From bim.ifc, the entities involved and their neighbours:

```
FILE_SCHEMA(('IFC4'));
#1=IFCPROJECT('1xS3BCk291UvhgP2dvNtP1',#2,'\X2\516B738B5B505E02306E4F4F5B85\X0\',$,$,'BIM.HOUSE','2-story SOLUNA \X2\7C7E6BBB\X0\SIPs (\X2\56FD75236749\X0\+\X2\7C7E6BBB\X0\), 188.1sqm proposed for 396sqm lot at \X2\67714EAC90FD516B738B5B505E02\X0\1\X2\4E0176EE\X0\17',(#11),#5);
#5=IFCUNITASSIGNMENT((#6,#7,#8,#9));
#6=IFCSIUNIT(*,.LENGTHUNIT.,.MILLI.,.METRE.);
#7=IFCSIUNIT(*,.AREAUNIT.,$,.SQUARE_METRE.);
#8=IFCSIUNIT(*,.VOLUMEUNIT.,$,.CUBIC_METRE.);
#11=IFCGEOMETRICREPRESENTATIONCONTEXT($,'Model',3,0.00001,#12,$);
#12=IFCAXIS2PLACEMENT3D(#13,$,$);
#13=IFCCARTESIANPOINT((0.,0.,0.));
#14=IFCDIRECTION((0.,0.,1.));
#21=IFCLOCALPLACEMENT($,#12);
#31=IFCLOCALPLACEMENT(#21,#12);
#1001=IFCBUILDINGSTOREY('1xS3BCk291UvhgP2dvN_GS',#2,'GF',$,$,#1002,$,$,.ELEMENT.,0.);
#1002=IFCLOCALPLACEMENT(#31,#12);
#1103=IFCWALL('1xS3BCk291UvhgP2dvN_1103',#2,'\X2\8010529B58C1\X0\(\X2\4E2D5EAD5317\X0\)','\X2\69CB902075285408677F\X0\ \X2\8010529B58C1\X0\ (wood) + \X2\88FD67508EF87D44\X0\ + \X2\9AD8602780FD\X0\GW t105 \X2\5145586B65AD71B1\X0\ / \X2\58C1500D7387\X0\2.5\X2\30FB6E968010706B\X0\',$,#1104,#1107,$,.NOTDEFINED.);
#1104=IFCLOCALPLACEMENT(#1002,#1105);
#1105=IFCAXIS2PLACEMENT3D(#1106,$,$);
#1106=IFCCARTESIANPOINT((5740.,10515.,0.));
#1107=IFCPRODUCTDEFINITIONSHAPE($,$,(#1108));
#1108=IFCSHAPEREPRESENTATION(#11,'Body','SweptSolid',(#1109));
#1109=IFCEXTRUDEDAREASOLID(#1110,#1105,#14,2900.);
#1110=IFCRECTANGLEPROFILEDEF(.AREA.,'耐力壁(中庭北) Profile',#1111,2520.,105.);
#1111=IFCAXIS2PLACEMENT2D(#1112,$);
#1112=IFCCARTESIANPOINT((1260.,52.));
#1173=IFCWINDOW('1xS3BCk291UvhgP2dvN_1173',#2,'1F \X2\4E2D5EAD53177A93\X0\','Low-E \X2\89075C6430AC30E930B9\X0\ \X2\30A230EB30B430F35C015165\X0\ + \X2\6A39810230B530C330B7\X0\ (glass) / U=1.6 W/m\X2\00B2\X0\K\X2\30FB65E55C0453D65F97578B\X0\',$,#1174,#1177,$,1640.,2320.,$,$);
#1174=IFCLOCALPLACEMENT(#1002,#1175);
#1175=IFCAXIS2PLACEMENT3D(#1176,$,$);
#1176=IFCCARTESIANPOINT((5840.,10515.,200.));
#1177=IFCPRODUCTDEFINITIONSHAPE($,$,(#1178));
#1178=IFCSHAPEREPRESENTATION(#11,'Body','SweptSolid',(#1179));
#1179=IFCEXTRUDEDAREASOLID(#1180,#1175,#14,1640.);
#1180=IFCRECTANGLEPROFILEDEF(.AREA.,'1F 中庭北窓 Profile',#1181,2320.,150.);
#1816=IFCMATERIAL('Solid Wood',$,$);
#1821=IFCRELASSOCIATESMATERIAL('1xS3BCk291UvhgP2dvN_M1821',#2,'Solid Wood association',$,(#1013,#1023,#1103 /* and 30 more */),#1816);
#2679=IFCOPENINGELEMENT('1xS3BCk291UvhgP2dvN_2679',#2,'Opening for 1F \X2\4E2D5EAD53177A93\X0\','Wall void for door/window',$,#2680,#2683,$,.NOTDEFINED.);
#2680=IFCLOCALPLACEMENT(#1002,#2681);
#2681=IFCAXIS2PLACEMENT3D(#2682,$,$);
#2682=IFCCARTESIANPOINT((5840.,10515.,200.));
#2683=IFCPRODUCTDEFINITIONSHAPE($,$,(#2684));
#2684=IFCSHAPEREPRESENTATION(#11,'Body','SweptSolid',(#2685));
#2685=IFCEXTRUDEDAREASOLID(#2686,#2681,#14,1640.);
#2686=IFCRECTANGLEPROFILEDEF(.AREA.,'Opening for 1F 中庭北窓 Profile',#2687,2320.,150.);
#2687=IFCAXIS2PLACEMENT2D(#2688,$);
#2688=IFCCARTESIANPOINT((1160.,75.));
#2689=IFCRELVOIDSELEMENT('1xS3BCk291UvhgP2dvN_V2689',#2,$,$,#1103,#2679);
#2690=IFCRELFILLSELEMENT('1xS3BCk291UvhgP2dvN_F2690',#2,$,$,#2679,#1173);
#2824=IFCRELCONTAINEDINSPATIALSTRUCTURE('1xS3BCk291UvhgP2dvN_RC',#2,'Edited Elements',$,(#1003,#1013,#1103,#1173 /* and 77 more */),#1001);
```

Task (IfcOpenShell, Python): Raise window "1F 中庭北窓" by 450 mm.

```python
import numpy as np
import ifcopenshell
import ifcopenshell.api.geometry
import ifcopenshell.util.placement
import ifcopenshell.util.unit

model = ifcopenshell.open("bim.ifc")
unit_scale = ifcopenshell.util.unit.calculate_unit_scale(model)

window = model.by_guid("1xS3BCk291UvhgP2dvN_1173")
opening = window.FillsVoids[0].RelatingOpeningElement
dz = 0.45 / unit_scale

shift = np.array([0.0, 0.0, dz])
# The window is not placed relative to its opening, so move both.
for product in (opening, window):
    matrix = ifcopenshell.util.placement.get_local_placement(product.ObjectPlacement)
    matrix[:3, 3] += shift
    ifcopenshell.api.geometry.edit_object_placement(model, product=product, matrix=matrix, is_si=False)

print(f"moved by {dz * unit_scale:+.3f} m")

model.write("bim_updated.ifc")
```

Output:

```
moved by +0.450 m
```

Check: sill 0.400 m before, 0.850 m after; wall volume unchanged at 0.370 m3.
